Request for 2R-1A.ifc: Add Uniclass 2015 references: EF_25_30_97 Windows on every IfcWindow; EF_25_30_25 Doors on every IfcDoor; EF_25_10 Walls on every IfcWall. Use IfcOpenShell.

First a look at what the model holds.

```python
import ifcopenshell

model = ifcopenshell.open("2R-1A.ifc")
print(model.schema)
print("classifications:", [c.Name for c in model.by_type("IfcClassification")])
for ifc_class in ("IfcDoor", "IfcRoof", "IfcStair", "IfcWall", "IfcWindow"):
    print(ifc_class, len(model.by_type(ifc_class)))
```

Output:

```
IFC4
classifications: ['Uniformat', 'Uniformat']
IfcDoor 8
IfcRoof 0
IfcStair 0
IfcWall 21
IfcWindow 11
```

```python
import ifcopenshell
import ifcopenshell.api.classification

model = ifcopenshell.open("2R-1A.ifc")

system = ifcopenshell.api.classification.add_classification(model, classification="Uniclass 2015")

codes = {
    "IfcWindow": ("EF_25_30_97", "Windows"),
    "IfcDoor": ("EF_25_30_25", "Doors"),
    "IfcWall": ("EF_25_10", "Walls"),
}
for ifc_class, (code, name) in codes.items():
    products = model.by_type(ifc_class)
    ifcopenshell.api.classification.add_reference(
        model, products=products, classification=system, identification=code, name=name
    )
    print(code, len(products))

model.write("2R-1A_rev.ifc")
```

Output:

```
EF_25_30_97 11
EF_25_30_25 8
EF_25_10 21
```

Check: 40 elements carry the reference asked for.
